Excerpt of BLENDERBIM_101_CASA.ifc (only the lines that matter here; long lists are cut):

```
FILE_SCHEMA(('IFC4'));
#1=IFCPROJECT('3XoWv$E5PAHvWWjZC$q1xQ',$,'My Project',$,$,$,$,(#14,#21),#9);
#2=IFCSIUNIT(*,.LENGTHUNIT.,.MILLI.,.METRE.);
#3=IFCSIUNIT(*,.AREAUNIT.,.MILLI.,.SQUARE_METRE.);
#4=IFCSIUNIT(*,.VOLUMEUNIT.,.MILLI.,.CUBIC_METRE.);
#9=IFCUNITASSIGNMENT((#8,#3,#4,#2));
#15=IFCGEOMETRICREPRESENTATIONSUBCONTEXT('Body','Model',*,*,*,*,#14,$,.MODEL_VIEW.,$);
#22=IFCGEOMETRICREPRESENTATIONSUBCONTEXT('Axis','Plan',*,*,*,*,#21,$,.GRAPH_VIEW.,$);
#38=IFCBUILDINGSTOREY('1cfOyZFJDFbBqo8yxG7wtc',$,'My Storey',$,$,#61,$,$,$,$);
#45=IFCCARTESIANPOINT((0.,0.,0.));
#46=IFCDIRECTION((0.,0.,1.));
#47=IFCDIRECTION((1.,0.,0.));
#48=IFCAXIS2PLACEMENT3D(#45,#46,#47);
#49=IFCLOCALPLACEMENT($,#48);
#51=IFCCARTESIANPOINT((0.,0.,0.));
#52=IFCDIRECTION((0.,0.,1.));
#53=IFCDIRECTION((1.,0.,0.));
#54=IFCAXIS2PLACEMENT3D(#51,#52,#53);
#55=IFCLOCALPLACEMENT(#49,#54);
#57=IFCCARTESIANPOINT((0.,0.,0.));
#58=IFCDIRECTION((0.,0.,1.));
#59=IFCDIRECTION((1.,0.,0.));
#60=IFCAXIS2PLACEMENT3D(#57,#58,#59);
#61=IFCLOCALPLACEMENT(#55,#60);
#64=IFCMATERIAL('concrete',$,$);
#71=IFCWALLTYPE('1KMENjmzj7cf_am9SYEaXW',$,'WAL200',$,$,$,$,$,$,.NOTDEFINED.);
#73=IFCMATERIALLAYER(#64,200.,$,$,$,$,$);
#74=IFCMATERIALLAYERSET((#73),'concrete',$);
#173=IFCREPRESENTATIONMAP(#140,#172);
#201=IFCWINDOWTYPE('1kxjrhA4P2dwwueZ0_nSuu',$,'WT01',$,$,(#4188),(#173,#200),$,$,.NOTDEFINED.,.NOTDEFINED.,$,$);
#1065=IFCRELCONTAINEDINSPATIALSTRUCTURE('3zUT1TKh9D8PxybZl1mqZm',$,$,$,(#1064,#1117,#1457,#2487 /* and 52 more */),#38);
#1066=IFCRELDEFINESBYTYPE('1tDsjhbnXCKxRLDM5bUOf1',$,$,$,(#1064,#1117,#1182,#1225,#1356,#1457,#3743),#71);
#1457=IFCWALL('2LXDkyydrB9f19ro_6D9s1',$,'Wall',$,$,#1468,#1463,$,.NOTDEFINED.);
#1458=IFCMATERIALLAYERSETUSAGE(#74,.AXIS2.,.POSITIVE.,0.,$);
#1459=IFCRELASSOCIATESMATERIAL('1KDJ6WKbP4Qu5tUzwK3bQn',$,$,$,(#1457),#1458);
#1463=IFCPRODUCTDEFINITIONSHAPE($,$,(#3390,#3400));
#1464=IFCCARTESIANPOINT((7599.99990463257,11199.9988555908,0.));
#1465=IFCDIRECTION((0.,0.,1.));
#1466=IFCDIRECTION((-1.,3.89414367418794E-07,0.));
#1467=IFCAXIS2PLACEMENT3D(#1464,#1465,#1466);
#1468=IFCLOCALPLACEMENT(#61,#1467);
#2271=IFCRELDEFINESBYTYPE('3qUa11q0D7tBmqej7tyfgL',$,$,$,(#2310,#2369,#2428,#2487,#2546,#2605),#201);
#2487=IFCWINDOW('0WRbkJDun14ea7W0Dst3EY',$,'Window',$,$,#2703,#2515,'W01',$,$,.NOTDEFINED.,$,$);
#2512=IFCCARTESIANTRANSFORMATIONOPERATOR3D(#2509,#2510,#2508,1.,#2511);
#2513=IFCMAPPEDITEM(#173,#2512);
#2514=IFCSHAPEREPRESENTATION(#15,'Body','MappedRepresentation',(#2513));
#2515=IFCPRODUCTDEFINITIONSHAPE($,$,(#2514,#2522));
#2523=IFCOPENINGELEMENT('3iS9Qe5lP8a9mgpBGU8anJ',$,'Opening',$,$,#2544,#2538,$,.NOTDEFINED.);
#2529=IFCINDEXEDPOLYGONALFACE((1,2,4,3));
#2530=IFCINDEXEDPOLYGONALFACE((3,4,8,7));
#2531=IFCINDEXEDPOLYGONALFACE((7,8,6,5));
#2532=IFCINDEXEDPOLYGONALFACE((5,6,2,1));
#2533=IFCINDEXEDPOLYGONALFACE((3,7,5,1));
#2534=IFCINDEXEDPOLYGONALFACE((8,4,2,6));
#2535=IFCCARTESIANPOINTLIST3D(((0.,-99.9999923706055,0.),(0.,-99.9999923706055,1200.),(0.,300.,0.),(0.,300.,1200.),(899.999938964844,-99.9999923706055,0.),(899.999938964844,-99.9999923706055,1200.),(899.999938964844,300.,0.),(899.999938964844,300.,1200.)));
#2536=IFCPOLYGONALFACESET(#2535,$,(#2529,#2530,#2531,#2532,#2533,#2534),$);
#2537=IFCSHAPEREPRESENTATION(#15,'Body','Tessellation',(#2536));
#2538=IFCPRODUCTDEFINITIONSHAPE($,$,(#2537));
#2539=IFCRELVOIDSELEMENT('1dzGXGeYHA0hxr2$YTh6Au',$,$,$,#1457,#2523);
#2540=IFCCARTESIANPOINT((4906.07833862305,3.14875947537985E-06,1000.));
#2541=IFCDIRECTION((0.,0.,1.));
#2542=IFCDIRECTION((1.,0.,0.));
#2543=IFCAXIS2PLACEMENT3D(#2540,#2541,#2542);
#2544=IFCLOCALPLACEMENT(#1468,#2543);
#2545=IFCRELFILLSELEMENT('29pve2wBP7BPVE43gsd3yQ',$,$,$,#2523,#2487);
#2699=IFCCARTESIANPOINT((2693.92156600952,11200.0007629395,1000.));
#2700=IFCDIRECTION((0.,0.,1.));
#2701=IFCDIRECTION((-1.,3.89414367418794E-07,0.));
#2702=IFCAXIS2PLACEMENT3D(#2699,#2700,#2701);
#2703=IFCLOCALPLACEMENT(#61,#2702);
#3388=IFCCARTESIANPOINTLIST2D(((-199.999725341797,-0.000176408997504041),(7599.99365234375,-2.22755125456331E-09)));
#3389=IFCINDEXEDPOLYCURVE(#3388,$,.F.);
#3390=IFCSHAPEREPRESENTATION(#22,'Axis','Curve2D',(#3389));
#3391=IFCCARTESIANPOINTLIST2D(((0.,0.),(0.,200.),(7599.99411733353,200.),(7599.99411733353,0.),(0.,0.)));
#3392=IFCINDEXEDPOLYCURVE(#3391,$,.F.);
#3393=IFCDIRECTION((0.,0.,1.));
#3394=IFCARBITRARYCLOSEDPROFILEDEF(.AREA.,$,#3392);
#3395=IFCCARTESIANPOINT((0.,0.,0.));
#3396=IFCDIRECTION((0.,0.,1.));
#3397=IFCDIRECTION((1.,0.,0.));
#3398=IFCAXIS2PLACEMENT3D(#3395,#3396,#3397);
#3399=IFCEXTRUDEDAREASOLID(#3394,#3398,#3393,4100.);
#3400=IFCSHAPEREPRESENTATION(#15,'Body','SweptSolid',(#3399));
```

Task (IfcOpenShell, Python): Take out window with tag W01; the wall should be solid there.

```python
import ifcopenshell
import ifcopenshell.api.feature
import ifcopenshell.api.root
import ifcopenshell.geom
import ifcopenshell.util.shape

model = ifcopenshell.open("BLENDERBIM_101_CASA.ifc")
settings = ifcopenshell.geom.settings()


def volume(element):
    """Net volume in cubic metres, openings subtracted."""
    shape = ifcopenshell.geom.create_shape(settings, element)
    return ifcopenshell.util.shape.get_volume(shape.geometry)


window = model.by_guid("0WRbkJDun14ea7W0Dst3EY")
opening = window.FillsVoids[0].RelatingOpeningElement
wall = opening.VoidsElements[0].RelatingBuildingElement
before = volume(wall)

ifcopenshell.api.root.remove_product(model, product=window)
ifcopenshell.api.feature.remove_feature(model, feature=opening)

after = volume(wall)

print(f"wall volume {before:.3f} -> {after:.3f} m3")

model.write("BLENDERBIM_101_CASA-out.ifc")
```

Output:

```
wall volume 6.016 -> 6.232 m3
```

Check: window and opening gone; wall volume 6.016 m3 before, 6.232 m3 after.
